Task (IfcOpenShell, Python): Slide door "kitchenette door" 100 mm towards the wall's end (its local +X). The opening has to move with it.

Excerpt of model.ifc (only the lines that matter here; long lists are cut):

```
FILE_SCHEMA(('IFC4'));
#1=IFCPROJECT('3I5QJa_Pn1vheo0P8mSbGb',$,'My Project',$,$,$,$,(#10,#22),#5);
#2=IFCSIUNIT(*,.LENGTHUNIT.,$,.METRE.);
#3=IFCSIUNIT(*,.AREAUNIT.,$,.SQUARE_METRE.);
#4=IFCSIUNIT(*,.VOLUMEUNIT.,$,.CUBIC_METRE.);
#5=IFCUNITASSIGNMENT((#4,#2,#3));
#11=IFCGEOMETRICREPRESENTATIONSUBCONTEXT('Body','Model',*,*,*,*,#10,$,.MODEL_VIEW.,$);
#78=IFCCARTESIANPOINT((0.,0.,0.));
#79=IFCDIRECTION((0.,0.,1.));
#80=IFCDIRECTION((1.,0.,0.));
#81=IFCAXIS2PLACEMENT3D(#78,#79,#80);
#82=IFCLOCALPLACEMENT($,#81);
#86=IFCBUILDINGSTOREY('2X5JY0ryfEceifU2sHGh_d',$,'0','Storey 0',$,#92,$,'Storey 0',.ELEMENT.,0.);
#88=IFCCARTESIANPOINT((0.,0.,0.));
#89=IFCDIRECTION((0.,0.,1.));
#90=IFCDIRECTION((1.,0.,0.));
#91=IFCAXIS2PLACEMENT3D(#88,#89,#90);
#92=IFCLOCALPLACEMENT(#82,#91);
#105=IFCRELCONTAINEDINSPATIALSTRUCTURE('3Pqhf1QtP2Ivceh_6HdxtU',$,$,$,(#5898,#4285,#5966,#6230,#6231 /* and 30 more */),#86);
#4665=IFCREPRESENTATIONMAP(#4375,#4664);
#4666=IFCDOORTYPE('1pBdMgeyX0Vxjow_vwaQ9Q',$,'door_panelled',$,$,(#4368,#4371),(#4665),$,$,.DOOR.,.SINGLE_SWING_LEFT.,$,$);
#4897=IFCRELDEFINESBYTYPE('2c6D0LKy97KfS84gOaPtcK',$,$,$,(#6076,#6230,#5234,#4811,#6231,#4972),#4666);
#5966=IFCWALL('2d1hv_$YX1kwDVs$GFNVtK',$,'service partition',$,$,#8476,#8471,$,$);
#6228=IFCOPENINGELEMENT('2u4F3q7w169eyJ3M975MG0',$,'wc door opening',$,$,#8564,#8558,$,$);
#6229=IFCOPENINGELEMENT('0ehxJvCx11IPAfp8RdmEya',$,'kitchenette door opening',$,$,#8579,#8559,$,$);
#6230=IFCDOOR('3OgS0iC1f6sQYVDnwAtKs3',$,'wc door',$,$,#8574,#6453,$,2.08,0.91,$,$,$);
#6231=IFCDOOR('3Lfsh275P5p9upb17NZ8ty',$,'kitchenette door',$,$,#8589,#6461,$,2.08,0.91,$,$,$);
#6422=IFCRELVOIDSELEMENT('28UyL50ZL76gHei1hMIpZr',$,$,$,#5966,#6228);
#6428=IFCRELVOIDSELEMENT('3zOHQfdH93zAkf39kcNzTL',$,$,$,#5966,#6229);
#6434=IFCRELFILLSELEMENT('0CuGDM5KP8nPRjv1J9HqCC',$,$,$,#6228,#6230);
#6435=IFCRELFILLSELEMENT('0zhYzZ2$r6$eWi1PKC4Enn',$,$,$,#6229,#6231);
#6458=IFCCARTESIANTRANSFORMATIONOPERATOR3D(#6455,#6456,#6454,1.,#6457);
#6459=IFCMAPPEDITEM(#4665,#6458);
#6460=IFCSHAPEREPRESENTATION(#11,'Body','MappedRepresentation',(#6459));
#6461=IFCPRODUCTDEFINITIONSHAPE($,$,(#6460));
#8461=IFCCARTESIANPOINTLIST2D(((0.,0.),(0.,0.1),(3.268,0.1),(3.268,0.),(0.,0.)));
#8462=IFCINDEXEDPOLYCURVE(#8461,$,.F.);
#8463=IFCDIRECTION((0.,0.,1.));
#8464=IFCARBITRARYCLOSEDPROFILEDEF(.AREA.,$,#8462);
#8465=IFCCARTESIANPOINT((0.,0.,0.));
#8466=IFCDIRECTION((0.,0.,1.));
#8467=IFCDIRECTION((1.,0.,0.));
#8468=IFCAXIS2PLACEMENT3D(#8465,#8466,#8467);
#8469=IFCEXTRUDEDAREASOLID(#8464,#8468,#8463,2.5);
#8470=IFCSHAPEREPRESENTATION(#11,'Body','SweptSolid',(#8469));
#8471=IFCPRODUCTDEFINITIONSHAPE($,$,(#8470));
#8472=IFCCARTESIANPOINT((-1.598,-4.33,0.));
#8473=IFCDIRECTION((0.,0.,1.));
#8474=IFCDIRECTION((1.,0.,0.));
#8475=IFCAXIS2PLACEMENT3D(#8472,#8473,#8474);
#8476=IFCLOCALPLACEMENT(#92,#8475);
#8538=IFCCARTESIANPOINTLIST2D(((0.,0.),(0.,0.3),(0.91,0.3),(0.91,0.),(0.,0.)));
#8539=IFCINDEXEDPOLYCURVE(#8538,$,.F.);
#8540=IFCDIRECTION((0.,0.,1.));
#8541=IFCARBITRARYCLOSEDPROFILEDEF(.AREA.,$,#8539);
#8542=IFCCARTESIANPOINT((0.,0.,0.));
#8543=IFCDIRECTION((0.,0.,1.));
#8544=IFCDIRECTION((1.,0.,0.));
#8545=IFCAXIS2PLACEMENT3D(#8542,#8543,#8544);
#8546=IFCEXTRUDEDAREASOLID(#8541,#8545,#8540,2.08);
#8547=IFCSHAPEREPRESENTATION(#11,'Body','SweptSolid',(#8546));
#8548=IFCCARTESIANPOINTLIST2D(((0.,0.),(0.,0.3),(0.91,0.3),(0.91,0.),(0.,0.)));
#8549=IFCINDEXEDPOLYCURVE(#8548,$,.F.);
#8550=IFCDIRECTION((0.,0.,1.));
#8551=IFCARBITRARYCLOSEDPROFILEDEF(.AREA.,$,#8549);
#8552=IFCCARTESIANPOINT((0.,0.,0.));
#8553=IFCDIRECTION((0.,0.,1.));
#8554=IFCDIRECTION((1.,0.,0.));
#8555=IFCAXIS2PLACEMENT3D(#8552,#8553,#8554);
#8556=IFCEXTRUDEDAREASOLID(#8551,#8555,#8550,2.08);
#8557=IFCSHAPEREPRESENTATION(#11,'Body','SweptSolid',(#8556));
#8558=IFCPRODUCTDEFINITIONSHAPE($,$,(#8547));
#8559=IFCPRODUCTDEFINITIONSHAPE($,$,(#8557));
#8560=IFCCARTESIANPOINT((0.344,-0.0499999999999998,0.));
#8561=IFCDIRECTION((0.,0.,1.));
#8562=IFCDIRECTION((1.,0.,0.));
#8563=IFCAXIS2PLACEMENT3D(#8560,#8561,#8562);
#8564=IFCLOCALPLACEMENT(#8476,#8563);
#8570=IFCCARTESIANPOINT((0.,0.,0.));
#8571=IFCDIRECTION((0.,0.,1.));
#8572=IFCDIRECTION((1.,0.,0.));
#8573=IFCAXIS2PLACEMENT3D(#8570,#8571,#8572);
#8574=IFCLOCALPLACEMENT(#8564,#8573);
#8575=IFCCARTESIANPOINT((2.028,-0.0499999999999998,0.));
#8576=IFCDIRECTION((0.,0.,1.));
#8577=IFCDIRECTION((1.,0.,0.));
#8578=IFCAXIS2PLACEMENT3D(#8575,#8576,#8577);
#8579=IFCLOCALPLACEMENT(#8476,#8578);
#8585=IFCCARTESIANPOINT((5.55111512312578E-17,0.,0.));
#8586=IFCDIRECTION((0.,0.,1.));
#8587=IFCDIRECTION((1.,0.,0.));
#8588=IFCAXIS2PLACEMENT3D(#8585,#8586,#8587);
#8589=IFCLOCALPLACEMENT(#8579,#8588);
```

```python
import ifcopenshell
import ifcopenshell.api.geometry
import ifcopenshell.util.placement
import ifcopenshell.util.unit

model = ifcopenshell.open("model.ifc")
unit_scale = ifcopenshell.util.unit.calculate_unit_scale(model)

door = model.by_guid("3Lfsh275P5p9upb17NZ8ty")
opening = door.FillsVoids[0].RelatingOpeningElement
wall = opening.VoidsElements[0].RelatingBuildingElement

wall_matrix = ifcopenshell.util.placement.get_local_placement(wall.ObjectPlacement)
shift = wall_matrix[:3, 0] * 0.1 / unit_scale
before = ifcopenshell.util.placement.get_local_placement(door.ObjectPlacement)[:3, 3].copy()

# The door is placed relative to its opening, so it follows when the opening moves.
matrix = ifcopenshell.util.placement.get_local_placement(opening.ObjectPlacement)
matrix[:3, 3] += shift
ifcopenshell.api.geometry.edit_object_placement(
    model, product=opening, matrix=matrix, is_si=False, should_transform_children=True
)

after = ifcopenshell.util.placement.get_local_placement(door.ObjectPlacement)[:3, 3]
print("door moved by", (after - before).round(3) + 0.0)

model.write("model-out.ifc")
```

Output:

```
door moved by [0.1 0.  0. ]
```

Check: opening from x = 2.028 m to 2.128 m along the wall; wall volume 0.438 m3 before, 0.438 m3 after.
